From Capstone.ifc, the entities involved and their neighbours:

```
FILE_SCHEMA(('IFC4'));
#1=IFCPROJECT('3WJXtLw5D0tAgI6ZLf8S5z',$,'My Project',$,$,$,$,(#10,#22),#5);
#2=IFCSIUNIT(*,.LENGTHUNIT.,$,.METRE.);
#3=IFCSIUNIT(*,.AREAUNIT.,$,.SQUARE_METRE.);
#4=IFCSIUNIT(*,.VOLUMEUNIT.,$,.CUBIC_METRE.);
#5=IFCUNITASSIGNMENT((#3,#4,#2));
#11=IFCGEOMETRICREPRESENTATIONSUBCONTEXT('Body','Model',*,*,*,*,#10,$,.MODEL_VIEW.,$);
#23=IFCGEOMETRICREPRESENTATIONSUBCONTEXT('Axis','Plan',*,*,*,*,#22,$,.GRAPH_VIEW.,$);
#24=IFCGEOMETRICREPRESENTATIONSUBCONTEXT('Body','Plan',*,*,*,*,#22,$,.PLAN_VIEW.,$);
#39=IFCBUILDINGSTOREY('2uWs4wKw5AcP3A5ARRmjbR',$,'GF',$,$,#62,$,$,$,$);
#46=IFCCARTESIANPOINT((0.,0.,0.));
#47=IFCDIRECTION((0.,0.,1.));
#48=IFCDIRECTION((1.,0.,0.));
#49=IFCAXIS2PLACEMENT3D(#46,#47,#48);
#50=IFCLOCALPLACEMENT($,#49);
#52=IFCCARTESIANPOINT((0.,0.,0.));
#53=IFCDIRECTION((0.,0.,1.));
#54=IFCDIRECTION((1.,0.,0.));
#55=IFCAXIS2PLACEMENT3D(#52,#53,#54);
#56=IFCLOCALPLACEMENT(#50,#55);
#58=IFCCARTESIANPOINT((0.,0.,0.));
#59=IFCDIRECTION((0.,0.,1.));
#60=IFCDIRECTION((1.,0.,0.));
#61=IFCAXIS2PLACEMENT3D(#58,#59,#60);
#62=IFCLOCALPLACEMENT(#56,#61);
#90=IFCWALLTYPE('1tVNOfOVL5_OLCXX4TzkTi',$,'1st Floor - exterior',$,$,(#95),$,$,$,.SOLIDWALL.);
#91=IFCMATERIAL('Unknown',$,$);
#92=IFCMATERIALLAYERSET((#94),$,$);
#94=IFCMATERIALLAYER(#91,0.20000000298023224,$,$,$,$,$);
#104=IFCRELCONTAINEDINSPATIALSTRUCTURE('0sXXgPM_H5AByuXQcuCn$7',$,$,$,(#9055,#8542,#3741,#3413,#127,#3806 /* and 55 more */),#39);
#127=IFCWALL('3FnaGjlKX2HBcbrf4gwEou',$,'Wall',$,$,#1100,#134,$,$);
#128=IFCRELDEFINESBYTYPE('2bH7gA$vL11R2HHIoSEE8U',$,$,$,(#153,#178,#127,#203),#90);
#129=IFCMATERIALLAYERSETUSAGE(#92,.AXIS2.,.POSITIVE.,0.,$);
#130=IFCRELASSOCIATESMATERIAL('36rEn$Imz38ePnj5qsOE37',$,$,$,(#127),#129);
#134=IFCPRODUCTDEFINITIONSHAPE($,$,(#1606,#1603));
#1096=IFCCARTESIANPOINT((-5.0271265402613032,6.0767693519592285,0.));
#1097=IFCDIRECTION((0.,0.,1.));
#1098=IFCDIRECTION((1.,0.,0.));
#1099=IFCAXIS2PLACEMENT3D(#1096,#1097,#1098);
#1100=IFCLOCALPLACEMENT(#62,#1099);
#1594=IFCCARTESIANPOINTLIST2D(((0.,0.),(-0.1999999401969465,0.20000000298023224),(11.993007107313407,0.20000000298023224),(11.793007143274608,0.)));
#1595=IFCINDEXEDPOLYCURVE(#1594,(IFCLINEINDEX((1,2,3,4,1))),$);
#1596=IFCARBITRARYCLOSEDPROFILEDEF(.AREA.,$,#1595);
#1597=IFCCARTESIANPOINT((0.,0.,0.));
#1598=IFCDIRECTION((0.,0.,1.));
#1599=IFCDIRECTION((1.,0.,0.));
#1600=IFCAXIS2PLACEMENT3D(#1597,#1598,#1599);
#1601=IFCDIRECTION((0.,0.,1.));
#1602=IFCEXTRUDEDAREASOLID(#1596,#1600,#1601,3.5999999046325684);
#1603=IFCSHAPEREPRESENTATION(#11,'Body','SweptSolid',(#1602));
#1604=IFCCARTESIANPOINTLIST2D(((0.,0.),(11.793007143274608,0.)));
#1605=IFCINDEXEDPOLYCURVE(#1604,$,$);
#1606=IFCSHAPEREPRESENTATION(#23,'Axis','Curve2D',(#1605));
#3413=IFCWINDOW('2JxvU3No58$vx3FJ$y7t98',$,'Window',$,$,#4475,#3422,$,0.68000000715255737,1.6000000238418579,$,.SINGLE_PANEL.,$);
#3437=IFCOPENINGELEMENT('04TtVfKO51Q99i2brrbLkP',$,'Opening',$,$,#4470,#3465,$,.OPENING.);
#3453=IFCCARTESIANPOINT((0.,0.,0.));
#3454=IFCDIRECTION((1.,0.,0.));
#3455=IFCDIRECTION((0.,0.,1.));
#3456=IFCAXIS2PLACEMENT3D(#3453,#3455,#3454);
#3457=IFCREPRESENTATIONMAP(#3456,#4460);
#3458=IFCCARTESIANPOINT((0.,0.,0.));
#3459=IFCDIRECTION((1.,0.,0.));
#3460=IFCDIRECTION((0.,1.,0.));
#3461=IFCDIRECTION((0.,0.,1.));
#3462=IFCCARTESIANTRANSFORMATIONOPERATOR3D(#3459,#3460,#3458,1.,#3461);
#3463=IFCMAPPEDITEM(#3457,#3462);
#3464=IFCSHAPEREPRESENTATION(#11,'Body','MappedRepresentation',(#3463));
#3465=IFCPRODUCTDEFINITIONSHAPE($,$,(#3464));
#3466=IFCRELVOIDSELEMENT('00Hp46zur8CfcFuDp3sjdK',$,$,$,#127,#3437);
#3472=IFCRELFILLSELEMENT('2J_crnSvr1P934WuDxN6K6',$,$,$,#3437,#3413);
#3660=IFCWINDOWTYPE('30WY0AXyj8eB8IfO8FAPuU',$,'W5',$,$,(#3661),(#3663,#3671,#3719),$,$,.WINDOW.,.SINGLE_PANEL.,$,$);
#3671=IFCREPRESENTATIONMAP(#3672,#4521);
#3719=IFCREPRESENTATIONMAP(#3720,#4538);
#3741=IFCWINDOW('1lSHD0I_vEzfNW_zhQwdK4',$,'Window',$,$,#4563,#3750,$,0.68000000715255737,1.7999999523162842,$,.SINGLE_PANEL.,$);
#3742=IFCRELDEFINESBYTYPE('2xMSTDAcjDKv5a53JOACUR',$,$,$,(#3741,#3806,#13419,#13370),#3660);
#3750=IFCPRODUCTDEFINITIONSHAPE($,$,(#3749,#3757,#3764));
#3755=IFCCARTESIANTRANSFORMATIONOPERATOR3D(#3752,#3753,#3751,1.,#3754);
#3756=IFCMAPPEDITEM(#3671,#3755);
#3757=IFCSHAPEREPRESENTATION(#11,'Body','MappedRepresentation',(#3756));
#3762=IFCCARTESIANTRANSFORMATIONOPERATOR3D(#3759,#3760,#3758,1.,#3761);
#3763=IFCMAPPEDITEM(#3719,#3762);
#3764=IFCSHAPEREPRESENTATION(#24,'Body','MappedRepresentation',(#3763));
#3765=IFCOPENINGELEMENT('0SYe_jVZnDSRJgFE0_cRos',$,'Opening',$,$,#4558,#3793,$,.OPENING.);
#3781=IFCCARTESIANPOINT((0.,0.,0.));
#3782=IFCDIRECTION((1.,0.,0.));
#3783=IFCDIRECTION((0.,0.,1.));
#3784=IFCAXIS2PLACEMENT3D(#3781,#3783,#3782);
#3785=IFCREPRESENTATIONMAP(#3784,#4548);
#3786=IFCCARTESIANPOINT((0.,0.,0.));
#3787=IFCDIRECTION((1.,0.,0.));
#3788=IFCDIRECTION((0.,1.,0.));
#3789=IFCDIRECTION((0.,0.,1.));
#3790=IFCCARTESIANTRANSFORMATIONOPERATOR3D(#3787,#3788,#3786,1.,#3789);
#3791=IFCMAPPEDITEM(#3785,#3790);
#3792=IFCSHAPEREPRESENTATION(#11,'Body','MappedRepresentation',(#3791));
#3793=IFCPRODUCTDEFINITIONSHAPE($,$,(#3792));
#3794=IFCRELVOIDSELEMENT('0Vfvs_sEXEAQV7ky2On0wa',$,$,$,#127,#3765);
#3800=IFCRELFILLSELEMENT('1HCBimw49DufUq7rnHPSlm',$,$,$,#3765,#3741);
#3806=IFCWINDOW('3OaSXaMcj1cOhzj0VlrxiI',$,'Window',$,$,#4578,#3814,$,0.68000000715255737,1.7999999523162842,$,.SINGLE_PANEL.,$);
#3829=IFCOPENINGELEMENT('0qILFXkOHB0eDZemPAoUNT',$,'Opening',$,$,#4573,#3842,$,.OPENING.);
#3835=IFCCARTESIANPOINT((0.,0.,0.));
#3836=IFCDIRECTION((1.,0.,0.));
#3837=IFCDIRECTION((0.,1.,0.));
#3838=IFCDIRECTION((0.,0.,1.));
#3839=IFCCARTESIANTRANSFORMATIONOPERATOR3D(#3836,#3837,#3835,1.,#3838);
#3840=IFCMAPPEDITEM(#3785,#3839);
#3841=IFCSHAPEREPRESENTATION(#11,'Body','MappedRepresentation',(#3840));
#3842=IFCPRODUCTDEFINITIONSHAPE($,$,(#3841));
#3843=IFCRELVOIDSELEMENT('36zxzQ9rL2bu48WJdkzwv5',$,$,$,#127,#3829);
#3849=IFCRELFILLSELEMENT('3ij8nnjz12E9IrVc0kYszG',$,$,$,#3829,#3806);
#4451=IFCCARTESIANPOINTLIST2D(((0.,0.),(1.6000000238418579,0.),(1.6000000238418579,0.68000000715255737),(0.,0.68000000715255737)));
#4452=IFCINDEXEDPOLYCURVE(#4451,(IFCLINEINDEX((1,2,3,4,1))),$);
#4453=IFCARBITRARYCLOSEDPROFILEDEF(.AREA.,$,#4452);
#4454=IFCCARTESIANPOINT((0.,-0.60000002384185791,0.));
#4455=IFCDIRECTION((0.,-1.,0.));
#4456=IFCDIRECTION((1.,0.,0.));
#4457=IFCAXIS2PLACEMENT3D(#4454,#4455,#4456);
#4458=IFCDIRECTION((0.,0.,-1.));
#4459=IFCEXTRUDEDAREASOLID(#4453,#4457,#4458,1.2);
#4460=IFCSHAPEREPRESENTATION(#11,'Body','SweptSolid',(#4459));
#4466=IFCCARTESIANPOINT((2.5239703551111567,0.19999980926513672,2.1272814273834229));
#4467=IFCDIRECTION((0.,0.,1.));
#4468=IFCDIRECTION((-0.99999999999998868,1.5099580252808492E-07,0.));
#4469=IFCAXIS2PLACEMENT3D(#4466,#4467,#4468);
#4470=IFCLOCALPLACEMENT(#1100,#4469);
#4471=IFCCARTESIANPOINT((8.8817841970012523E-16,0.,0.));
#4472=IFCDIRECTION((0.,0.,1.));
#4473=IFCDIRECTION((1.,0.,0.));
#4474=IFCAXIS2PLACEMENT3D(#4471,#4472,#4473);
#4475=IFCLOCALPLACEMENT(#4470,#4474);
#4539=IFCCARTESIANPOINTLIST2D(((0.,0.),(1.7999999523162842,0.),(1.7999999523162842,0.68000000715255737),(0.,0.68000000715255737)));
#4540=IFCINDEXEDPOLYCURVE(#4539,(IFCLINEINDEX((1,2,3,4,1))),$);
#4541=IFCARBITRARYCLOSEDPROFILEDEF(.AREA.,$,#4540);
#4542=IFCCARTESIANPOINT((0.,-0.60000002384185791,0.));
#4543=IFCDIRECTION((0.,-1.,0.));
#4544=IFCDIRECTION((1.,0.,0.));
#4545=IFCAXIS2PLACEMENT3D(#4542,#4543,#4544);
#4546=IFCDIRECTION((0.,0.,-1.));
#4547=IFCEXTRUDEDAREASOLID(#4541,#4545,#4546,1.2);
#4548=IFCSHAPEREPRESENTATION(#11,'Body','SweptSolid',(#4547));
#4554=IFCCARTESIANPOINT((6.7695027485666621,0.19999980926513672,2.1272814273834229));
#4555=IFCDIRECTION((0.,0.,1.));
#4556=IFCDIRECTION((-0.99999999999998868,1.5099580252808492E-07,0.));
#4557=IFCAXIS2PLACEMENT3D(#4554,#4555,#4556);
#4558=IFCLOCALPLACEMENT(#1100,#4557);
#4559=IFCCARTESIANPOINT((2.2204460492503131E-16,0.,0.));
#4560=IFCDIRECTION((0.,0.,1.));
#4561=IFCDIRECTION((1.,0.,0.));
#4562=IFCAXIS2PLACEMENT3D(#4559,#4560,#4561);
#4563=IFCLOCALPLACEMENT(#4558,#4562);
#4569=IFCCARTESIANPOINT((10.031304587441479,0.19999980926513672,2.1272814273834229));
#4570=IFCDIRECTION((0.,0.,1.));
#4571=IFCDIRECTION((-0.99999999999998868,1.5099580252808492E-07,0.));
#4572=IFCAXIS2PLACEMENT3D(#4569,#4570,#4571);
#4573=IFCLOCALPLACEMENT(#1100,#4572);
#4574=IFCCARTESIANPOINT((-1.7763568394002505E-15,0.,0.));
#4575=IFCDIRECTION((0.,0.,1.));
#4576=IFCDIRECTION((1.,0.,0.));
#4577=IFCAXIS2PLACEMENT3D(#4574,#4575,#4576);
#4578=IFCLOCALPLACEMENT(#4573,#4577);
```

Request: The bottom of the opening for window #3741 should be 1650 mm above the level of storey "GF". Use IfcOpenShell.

```python
import numpy as np
import ifcopenshell
import ifcopenshell.api.geometry
import ifcopenshell.geom
import ifcopenshell.util.element
import ifcopenshell.util.placement
import ifcopenshell.util.shape
import ifcopenshell.util.unit

model = ifcopenshell.open("Capstone.ifc")
unit_scale = ifcopenshell.util.unit.calculate_unit_scale(model)

window = model.by_id(3741)
opening = window.FillsVoids[0].RelatingOpeningElement
storey = ifcopenshell.util.element.get_container(window, ifc_class="IfcBuildingStorey")
level = ifcopenshell.util.placement.get_local_placement(storey.ObjectPlacement)[2, 3]

# The opening's origin need not be at the sill, so measure its lowest point.
shape = ifcopenshell.geom.create_shape(ifcopenshell.geom.settings(), opening)
bottom = ifcopenshell.util.shape.get_shape_bottom_elevation(shape, shape.geometry) / unit_scale
dz = level + 1.65 / unit_scale - bottom

shift = np.array([0.0, 0.0, dz])
# The window is placed relative to its opening, so it follows when the opening moves.
matrix = ifcopenshell.util.placement.get_local_placement(opening.ObjectPlacement)
matrix[:3, 3] += shift
ifcopenshell.api.geometry.edit_object_placement(
    model, product=opening, matrix=matrix, is_si=False, should_transform_children=True
)

print(f"moved by {dz * unit_scale:+.3f} m")

model.write("Capstone_edited.ifc")
```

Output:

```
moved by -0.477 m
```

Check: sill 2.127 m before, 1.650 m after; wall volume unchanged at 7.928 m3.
